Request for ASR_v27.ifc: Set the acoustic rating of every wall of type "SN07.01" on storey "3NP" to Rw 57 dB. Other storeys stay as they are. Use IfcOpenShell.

First a look at what the model holds.

```python
import ifcopenshell
import ifcopenshell.util.element

model = ifcopenshell.open("ASR_v27.ifc")
print(model.schema)
storey = next(s for s in model.by_type("IfcBuildingStorey") if s.Name == "3NP")
walls = [e for e in ifcopenshell.util.element.get_decomposition(storey) if e.is_a("IfcWall")]
seen = {}
for e in walls:
    element_type = ifcopenshell.util.element.get_type(e)
    key = (element_type.Name if element_type != e and element_type else None, ifcopenshell.util.element.get_pset(e, "Pset_WallCommon", "AcousticRating"))
    seen[key] = seen.get(key, 0) + 1
for (name, value), count in sorted(seen.items(), key=str):
    print(count, "x", name, "|", value)
```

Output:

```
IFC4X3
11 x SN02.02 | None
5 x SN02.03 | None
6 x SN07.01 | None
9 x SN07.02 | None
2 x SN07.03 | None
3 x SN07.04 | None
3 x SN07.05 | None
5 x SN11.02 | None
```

```python
import ifcopenshell
import ifcopenshell.api.pset
import ifcopenshell.util.element

model = ifcopenshell.open("ASR_v27.ifc")

storey = next(s for s in model.by_type("IfcBuildingStorey") if s.Name == "3NP")
walls = [e for e in ifcopenshell.util.element.get_decomposition(storey) if e.is_a("IfcWall")]

count = 0
for e in walls:
    element_type = ifcopenshell.util.element.get_type(e)
    if element_type in (None, e) or element_type.Name != "SN07.01":
        continue
    # add_pset returns the element's existing set when there is one.
    pset = ifcopenshell.api.pset.add_pset(model, product=e, name="Pset_WallCommon")
    ifcopenshell.api.pset.edit_pset(model, pset=pset, properties={"AcousticRating": "Rw 57 dB"})
    count += 1

print(count, "walls updated")

model.write("ASR_v27_v2.ifc")
```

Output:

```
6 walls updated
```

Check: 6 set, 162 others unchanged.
